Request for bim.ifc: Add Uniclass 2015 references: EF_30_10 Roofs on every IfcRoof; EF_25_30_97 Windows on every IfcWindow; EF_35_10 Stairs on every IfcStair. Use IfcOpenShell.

First a look at what the model holds.

```python
import ifcopenshell

model = ifcopenshell.open("bim.ifc")
print(model.schema)
print("classifications:", [c.Name for c in model.by_type("IfcClassification")])
for ifc_class in ("IfcDoor", "IfcRoof", "IfcStair", "IfcWall", "IfcWindow"):
    print(ifc_class, len(model.by_type(ifc_class)))
```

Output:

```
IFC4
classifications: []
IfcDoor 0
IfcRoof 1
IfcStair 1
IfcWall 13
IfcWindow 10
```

```python
import ifcopenshell
import ifcopenshell.api.classification

model = ifcopenshell.open("bim.ifc")

system = ifcopenshell.api.classification.add_classification(model, classification="Uniclass 2015")

codes = {
    "IfcRoof": ("EF_30_10", "Roofs"),
    "IfcWindow": ("EF_25_30_97", "Windows"),
    "IfcStair": ("EF_35_10", "Stairs"),
}
for ifc_class, (code, name) in codes.items():
    products = model.by_type(ifc_class)
    ifcopenshell.api.classification.add_reference(
        model, products=products, classification=system, identification=code, name=name
    )
    print(code, len(products))

model.write("bim_rev.ifc")
```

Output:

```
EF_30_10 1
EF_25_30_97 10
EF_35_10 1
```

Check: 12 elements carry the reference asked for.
